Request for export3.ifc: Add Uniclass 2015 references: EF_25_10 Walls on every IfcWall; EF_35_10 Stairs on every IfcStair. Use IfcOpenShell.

First a look at what the model holds.

```python
import ifcopenshell

model = ifcopenshell.open("export3.ifc")
print(model.schema)
print("classifications:", [c.Name for c in model.by_type("IfcClassification")])
for ifc_class in ("IfcDoor", "IfcRoof", "IfcStair", "IfcWall", "IfcWindow"):
    print(ifc_class, len(model.by_type(ifc_class)))
```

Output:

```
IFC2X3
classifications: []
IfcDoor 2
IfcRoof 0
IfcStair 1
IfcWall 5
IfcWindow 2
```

```python
import ifcopenshell
import ifcopenshell.api.classification

model = ifcopenshell.open("export3.ifc")

# IFC2X3 requires Source and Edition and has no link from the project to the system.
system = model.create_entity("IfcClassification", Source="NBS", Edition="2015", Name="Uniclass 2015")

codes = {
    "IfcWall": ("EF_25_10", "Walls"),
    "IfcStair": ("EF_35_10", "Stairs"),
}
for ifc_class, (code, name) in codes.items():
    products = model.by_type(ifc_class)
    ifcopenshell.api.classification.add_reference(
        model, products=products, classification=system, identification=code, name=name
    )
    print(code, len(products))

model.write("export3_v2.ifc")
```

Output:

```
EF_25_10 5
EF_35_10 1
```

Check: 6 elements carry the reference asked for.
